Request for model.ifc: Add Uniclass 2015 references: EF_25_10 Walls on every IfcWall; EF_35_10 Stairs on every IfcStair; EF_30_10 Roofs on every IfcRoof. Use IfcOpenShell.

First a look at what the model holds.

```python
import ifcopenshell

model = ifcopenshell.open("model.ifc")
print(model.schema)
print("classifications:", [c.Name for c in model.by_type("IfcClassification")])
for ifc_class in ("IfcDoor", "IfcRoof", "IfcStair", "IfcWall", "IfcWindow"):
    print(ifc_class, len(model.by_type(ifc_class)))
```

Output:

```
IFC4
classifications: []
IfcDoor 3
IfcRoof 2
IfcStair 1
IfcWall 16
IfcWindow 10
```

```python
import ifcopenshell
import ifcopenshell.api.classification

model = ifcopenshell.open("model.ifc")

system = ifcopenshell.api.classification.add_classification(model, classification="Uniclass 2015")

codes = {
    "IfcWall": ("EF_25_10", "Walls"),
    "IfcStair": ("EF_35_10", "Stairs"),
    "IfcRoof": ("EF_30_10", "Roofs"),
}
for ifc_class, (code, name) in codes.items():
    products = model.by_type(ifc_class)
    ifcopenshell.api.classification.add_reference(
        model, products=products, classification=system, identification=code, name=name
    )
    print(code, len(products))

model.write("model_v2.ifc")
```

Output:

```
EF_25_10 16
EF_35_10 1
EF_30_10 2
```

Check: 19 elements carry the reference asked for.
